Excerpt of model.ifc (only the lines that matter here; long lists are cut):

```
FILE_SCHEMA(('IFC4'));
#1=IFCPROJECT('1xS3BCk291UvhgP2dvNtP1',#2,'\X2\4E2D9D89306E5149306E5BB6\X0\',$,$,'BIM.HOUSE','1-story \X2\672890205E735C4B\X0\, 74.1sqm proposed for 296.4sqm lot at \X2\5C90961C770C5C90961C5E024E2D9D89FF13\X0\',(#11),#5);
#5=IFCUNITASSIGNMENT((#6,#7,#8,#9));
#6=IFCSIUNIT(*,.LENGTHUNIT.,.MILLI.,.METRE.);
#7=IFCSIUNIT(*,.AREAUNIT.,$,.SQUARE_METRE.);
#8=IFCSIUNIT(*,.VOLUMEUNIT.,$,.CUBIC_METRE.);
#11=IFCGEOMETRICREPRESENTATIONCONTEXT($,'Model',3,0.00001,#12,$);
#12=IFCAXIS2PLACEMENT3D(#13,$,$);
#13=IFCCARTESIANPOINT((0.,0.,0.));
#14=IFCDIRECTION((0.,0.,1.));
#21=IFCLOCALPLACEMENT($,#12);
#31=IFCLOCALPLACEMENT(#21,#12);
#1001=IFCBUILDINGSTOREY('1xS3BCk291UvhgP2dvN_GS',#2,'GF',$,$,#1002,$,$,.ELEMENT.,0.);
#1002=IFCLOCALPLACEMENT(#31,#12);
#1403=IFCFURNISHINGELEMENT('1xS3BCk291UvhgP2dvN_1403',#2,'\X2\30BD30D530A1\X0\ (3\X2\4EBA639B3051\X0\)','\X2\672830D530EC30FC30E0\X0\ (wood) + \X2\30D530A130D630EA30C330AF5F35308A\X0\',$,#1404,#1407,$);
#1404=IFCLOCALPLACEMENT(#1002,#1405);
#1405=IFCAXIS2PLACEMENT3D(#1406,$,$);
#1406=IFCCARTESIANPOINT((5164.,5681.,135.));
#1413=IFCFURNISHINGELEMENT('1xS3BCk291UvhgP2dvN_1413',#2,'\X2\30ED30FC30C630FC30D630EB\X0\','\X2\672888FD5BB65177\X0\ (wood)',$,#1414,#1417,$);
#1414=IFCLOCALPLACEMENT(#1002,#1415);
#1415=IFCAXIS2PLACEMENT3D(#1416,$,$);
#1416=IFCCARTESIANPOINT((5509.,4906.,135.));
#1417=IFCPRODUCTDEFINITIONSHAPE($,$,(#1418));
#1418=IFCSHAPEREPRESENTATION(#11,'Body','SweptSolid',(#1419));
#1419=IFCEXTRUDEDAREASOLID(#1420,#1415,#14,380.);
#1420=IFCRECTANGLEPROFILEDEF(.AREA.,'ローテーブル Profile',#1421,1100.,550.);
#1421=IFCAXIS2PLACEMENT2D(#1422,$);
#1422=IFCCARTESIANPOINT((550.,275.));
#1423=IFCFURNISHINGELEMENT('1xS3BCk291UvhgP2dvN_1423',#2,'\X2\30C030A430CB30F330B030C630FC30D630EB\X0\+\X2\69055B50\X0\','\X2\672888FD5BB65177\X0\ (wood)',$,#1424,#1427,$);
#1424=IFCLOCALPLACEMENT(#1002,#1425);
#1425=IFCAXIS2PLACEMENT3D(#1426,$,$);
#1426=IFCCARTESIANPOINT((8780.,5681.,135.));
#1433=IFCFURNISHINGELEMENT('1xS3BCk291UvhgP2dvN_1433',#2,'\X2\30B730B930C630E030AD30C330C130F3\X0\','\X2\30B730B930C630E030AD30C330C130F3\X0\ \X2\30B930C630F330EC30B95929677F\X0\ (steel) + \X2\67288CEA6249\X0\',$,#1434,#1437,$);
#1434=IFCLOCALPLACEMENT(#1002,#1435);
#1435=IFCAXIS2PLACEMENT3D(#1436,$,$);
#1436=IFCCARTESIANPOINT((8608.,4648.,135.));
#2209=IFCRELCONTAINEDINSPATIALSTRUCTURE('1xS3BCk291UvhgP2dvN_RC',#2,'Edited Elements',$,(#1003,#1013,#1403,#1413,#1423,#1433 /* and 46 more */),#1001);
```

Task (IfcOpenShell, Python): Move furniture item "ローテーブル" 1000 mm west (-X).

```python
import ifcopenshell
import ifcopenshell.api.geometry
import ifcopenshell.util.placement
import ifcopenshell.util.unit

model = ifcopenshell.open("model.ifc")
unit_scale = ifcopenshell.util.unit.calculate_unit_scale(model)

item = model.by_guid("1xS3BCk291UvhgP2dvN_1413")
matrix = ifcopenshell.util.placement.get_local_placement(item.ObjectPlacement)
matrix[0, 3] -= 1 / unit_scale
ifcopenshell.api.geometry.edit_object_placement(model, product=item, matrix=matrix, is_si=False)

print(ifcopenshell.util.placement.get_local_placement(item.ObjectPlacement).round(3) + 0.0)

model.write("model-out.ifc")
```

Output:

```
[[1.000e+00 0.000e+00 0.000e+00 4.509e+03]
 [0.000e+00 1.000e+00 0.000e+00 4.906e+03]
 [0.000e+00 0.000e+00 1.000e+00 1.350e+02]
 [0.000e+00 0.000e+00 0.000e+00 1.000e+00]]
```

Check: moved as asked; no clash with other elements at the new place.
